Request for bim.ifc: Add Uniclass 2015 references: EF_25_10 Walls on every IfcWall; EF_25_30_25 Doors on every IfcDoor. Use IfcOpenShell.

First a look at what the model holds.

```python
import ifcopenshell

model = ifcopenshell.open("bim.ifc")
print(model.schema)
print("classifications:", [c.Name for c in model.by_type("IfcClassification")])
for ifc_class in ("IfcDoor", "IfcRoof", "IfcStair", "IfcWall", "IfcWindow"):
    print(ifc_class, len(model.by_type(ifc_class)))
```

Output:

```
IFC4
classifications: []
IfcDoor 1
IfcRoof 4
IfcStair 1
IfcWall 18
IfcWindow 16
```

```python
import ifcopenshell
import ifcopenshell.api.classification

model = ifcopenshell.open("bim.ifc")

system = ifcopenshell.api.classification.add_classification(model, classification="Uniclass 2015")

codes = {
    "IfcWall": ("EF_25_10", "Walls"),
    "IfcDoor": ("EF_25_30_25", "Doors"),
}
for ifc_class, (code, name) in codes.items():
    products = model.by_type(ifc_class)
    ifcopenshell.api.classification.add_reference(
        model, products=products, classification=system, identification=code, name=name
    )
    print(code, len(products))

model.write("bim_v2.ifc")
```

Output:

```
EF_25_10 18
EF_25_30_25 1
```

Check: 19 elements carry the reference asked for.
